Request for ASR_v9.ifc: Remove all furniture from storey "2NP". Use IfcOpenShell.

First a look at what the model holds.

```python
import ifcopenshell
import ifcopenshell.util.element

model = ifcopenshell.open("ASR_v9.ifc")
print(model.schema)
storey = next(s for s in model.by_type("IfcBuildingStorey") if s.Name == "2NP")
furniture = [e for e in ifcopenshell.util.element.get_decomposition(storey) if e.is_a("IfcFurnishingElement")]
seen = {}
for e in furniture:
    element_type = ifcopenshell.util.element.get_type(e)
    name = element_type.Name if element_type not in (None, e) else None
    seen[name] = seen.get(name, 0) + 1
for name, count in sorted(seen.items(), key=str):
    print(count, "x", name)
```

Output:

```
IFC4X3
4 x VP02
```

```python
import ifcopenshell
import ifcopenshell.api.root
import ifcopenshell.util.element

model = ifcopenshell.open("ASR_v9.ifc")

storey = next(s for s in model.by_type("IfcBuildingStorey") if s.Name == "2NP")
furniture = [e for e in ifcopenshell.util.element.get_decomposition(storey) if e.is_a("IfcFurnishingElement")]

for e in furniture:
    ifcopenshell.api.root.remove_product(model, product=e)
print(len(furniture), "removed")

model.write("ASR_v9_edited.ifc")
```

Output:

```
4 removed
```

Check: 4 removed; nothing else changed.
